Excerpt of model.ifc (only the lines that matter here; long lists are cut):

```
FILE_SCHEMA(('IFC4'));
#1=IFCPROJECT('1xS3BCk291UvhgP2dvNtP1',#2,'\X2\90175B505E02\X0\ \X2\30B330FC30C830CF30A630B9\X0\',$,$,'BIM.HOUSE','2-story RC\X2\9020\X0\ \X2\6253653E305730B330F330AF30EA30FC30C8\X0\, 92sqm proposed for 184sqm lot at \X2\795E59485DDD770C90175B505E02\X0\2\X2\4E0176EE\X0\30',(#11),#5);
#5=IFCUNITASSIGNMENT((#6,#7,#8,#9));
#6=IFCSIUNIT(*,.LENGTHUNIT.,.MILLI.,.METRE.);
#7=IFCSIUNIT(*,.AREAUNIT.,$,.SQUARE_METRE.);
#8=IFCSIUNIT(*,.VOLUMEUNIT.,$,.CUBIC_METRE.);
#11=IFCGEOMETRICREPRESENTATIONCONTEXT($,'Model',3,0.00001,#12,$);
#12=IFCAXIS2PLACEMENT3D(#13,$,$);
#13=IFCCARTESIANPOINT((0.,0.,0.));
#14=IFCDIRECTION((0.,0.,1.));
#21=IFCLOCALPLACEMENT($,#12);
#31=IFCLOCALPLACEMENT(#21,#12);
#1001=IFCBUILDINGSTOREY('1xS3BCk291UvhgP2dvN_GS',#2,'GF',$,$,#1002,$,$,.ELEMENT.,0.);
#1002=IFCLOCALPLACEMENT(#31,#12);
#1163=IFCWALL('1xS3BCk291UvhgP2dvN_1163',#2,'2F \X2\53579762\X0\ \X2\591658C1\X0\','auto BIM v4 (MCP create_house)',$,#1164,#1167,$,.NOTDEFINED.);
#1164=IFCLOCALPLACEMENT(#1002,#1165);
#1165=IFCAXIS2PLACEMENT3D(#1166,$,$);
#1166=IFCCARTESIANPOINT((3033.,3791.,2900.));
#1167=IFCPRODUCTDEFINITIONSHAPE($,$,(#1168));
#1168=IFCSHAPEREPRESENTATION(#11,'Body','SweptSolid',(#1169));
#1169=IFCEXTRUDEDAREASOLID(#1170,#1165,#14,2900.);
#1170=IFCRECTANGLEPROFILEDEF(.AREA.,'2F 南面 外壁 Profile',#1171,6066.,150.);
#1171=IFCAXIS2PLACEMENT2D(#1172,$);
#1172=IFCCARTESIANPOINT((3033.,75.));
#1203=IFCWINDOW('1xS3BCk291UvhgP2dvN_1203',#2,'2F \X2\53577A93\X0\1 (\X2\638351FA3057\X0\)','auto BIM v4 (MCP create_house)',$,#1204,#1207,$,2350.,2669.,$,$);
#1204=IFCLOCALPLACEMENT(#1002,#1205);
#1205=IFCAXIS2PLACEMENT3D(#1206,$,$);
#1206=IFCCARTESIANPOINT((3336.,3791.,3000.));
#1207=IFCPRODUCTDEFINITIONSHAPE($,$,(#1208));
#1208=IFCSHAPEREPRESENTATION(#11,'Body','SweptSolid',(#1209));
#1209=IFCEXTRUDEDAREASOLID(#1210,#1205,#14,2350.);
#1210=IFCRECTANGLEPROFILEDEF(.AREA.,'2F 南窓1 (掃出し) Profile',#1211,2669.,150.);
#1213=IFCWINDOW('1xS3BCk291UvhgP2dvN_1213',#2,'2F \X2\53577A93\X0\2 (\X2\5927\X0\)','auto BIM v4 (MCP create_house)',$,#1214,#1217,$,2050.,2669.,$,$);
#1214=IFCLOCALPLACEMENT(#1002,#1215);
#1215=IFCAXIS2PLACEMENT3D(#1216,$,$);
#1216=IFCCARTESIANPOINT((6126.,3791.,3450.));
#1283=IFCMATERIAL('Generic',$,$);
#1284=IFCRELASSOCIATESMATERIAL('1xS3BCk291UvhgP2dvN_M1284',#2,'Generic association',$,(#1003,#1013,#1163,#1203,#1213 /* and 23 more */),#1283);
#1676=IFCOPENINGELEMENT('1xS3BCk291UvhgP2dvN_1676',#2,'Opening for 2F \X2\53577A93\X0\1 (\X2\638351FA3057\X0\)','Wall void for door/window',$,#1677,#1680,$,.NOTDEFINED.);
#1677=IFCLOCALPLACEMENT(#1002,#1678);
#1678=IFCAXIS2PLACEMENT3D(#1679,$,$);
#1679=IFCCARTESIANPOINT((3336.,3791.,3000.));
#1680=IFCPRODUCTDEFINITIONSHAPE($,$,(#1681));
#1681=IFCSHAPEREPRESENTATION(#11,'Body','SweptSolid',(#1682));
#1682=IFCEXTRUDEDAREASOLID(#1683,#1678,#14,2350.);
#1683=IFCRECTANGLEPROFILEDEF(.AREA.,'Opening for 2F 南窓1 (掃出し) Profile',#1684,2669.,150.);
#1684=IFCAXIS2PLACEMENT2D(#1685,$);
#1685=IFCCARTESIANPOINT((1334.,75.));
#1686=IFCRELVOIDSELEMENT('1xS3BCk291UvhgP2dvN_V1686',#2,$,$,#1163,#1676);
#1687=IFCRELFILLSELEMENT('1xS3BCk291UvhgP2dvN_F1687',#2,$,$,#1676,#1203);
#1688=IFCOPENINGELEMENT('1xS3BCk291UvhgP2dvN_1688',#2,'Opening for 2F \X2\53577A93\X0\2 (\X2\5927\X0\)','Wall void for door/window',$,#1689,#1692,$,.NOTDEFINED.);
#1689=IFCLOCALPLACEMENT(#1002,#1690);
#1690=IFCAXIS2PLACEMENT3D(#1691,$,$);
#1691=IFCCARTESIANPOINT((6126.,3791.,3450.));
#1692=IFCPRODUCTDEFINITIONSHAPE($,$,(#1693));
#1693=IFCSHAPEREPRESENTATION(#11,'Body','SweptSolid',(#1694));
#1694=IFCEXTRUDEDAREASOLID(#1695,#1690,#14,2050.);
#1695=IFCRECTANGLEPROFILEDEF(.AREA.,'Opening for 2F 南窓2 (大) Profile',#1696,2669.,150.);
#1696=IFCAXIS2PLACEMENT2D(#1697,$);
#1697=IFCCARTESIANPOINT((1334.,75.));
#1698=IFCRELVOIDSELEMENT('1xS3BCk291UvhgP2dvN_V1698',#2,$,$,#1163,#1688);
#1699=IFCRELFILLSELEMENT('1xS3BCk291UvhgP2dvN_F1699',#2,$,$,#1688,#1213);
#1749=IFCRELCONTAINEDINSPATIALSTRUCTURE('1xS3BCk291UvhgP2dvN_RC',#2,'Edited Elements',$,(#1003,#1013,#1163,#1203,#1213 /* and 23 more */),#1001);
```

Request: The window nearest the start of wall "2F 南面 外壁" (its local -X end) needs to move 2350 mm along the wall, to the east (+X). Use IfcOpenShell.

```python
import ifcopenshell
import ifcopenshell.api.geometry
import ifcopenshell.util.placement
import ifcopenshell.util.unit

model = ifcopenshell.open("model.ifc")
unit_scale = ifcopenshell.util.unit.calculate_unit_scale(model)

window = model.by_guid("1xS3BCk291UvhgP2dvN_1203")
opening = window.FillsVoids[0].RelatingOpeningElement
wall = opening.VoidsElements[0].RelatingBuildingElement

wall_matrix = ifcopenshell.util.placement.get_local_placement(wall.ObjectPlacement)
shift = wall_matrix[:3, 0] * 2.35 / unit_scale
before = ifcopenshell.util.placement.get_local_placement(window.ObjectPlacement)[:3, 3].copy()

# The window is not placed relative to its opening, so move both.
for product in (opening, window):
    matrix = ifcopenshell.util.placement.get_local_placement(product.ObjectPlacement)
    matrix[:3, 3] += shift
    ifcopenshell.api.geometry.edit_object_placement(model, product=product, matrix=matrix, is_si=False)

after = ifcopenshell.util.placement.get_local_placement(window.ObjectPlacement)[:3, 3]
print("window moved by", (after - before).round(3) + 0.0)

model.write("model-out.ifc")
```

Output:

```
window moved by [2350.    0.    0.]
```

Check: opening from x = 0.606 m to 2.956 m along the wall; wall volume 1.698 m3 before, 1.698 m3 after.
